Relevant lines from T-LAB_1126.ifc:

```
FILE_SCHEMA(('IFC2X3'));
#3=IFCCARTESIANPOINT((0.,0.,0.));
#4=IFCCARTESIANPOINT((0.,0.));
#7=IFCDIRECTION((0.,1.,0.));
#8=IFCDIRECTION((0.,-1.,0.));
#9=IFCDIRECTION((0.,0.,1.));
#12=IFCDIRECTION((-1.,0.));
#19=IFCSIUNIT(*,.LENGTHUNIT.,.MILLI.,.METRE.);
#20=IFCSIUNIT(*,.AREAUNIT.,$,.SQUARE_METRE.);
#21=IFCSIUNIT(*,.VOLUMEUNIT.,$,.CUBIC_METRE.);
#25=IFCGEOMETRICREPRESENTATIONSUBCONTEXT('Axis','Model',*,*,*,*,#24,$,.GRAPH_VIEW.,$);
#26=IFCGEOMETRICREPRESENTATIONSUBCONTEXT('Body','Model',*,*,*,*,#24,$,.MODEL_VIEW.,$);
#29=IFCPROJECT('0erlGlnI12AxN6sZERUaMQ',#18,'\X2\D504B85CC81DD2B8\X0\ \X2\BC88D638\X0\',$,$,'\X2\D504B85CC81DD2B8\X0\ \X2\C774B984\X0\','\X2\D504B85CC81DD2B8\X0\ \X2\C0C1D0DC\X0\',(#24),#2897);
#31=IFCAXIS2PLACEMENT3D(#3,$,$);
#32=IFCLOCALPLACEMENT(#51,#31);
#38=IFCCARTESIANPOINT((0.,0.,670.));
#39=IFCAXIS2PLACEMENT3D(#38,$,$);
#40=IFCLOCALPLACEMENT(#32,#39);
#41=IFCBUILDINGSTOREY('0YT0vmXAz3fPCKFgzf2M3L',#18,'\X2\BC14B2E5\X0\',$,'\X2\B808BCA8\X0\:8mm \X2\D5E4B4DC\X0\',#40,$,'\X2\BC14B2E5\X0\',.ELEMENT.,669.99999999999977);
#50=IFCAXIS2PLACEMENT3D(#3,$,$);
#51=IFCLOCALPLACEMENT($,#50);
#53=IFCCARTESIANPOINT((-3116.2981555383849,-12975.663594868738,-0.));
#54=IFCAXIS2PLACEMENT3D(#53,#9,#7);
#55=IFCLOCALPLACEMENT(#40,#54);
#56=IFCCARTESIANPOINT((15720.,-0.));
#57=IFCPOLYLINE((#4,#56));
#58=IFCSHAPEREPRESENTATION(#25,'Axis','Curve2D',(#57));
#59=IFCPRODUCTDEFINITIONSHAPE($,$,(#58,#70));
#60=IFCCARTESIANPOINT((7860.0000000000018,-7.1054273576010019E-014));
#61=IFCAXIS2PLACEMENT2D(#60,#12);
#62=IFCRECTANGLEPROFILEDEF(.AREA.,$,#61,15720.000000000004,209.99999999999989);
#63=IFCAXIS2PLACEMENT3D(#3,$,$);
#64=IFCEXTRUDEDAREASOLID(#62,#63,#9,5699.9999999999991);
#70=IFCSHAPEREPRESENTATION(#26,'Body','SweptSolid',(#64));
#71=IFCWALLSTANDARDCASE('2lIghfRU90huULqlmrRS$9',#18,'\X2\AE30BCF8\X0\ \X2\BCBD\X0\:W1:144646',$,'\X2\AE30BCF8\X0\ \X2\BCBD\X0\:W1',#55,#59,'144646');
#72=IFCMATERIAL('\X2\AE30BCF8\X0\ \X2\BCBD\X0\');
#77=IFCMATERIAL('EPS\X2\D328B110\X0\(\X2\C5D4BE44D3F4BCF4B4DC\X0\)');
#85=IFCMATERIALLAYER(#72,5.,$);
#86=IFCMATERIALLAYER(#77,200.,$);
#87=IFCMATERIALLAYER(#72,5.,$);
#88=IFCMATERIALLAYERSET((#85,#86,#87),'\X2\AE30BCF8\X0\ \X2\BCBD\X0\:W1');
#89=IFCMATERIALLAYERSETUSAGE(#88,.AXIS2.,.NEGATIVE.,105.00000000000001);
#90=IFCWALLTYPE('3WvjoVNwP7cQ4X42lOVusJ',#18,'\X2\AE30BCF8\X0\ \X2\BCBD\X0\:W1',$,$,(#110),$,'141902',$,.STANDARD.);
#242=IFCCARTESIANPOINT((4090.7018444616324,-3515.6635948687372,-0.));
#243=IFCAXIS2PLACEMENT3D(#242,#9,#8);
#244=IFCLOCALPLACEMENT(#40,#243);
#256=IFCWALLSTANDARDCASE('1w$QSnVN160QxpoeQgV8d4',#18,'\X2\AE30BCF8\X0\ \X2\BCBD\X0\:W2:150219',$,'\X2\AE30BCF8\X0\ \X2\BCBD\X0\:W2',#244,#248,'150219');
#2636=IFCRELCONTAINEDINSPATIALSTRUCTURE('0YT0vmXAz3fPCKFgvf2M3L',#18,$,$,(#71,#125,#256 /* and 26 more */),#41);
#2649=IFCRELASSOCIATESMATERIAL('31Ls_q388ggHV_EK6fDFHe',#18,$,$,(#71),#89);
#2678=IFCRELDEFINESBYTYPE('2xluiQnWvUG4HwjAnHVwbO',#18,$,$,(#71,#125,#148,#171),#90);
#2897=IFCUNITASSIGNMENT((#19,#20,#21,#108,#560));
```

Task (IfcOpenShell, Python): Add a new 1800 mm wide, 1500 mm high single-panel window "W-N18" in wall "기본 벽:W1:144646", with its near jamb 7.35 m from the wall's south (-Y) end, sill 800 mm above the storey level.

```python
import numpy as np
import ifcopenshell
import ifcopenshell.api.feature
import ifcopenshell.api.geometry
import ifcopenshell.api.root
import ifcopenshell.api.spatial
import ifcopenshell.api.type
import ifcopenshell.geom
import ifcopenshell.util.element
import ifcopenshell.util.placement
import ifcopenshell.util.representation
import ifcopenshell.util.shape
import ifcopenshell.util.unit

model = ifcopenshell.open("T-LAB_1126.ifc")
unit_scale = ifcopenshell.util.unit.calculate_unit_scale(model)
settings = ifcopenshell.geom.settings()


def volume(element):
    """Net volume in cubic metres, openings subtracted."""
    shape = ifcopenshell.geom.create_shape(settings, element)
    return ifcopenshell.util.shape.get_volume(shape.geometry)


wall = model.by_guid("2lIghfRU90huULqlmrRS$9")
storey = ifcopenshell.util.element.get_container(wall, ifc_class="IfcBuildingStorey")
context = ifcopenshell.util.representation.get_context(model, "Model", "Body", "MODEL_VIEW")
before = volume(wall)

width, height, from_end, sill = 1.8, 1.5, 7.35, 0.8  # metres

# The wall runs along its own X axis, and the end named is its -X end.
wall_shape = ifcopenshell.geom.create_shape(settings, wall)
x, y, z = ifcopenshell.util.shape.get_vertices(wall_shape.geometry).T
start = x.min() + from_end
face, thickness = float(y.min()), float(y.max() - y.min())
wall_matrix = ifcopenshell.util.placement.get_local_placement(wall.ObjectPlacement)
level = ifcopenshell.util.placement.get_local_placement(storey.ObjectPlacement)[2, 3]


def in_wall(x, y):
    """Placement at x, y metres in the wall's axes, at sill height."""
    matrix = wall_matrix.copy()
    matrix[:, 3] = wall_matrix @ np.array([x / unit_scale, y / unit_scale, 0.0, 1.0])
    matrix[2, 3] = level + sill / unit_scale
    return matrix


# Opening: a box that overshoots both wall faces by 50 mm.
opening = ifcopenshell.api.root.create_entity(model, ifc_class="IfcOpeningElement")
box = ifcopenshell.api.geometry.add_wall_representation(
    model, context=context, length=width, height=height, thickness=thickness + 0.1
)
ifcopenshell.api.geometry.assign_representation(model, product=opening, representation=box)
ifcopenshell.api.geometry.edit_object_placement(model, product=opening, matrix=in_wall(start, face - 0.05), is_si=False)
ifcopenshell.api.feature.add_feature(model, feature=opening, element=wall)

window = ifcopenshell.api.root.create_entity(model, ifc_class="IfcWindow", name="W-N18")
window.OverallWidth, window.OverallHeight = width / unit_scale, height / unit_scale
body = ifcopenshell.api.geometry.add_window_representation(
    model,
    context=context,
    overall_width=window.OverallWidth,
    overall_height=window.OverallHeight,
    partition_type="SINGLE_PANEL",
)
ifcopenshell.api.geometry.assign_representation(model, product=window, representation=body)
ifcopenshell.api.spatial.assign_container(model, products=[window], relating_structure=storey)
fills = ifcopenshell.api.feature.add_filling(model, opening=opening, element=window)
fills.OwnerHistory = window.OwnerHistory  # required in IFC2X3

# IFC2X3 keeps the operation on the window style.
style = ifcopenshell.api.root.create_entity(model, ifc_class="IfcWindowStyle", name="W-N18")
style.OperationType, style.ConstructionType = "SINGLE_PANEL", "NOTDEFINED"
style.ParameterTakesPrecedence = style.Sizeable = False
ifcopenshell.api.type.assign_type(model, related_objects=[window], relating_type=style)

# Centre the window in the wall's thickness.
ifcopenshell.api.geometry.edit_object_placement(model, product=window, matrix=in_wall(start, face), is_si=False)
window_shape = ifcopenshell.geom.create_shape(settings, window)
depth = ifcopenshell.util.shape.get_vertices(window_shape.geometry)[:, 1]
offset = face + thickness / 2 - (depth.min() + depth.max()) / 2
ifcopenshell.api.geometry.edit_object_placement(model, product=window, matrix=in_wall(start, offset), is_si=False)

after = volume(wall)

print(f"wall volume {before:.3f} -> {after:.3f} m3")

model.write("T-LAB_1126_rev.ifc")
```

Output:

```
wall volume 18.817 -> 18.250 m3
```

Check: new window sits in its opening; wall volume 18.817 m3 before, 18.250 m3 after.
